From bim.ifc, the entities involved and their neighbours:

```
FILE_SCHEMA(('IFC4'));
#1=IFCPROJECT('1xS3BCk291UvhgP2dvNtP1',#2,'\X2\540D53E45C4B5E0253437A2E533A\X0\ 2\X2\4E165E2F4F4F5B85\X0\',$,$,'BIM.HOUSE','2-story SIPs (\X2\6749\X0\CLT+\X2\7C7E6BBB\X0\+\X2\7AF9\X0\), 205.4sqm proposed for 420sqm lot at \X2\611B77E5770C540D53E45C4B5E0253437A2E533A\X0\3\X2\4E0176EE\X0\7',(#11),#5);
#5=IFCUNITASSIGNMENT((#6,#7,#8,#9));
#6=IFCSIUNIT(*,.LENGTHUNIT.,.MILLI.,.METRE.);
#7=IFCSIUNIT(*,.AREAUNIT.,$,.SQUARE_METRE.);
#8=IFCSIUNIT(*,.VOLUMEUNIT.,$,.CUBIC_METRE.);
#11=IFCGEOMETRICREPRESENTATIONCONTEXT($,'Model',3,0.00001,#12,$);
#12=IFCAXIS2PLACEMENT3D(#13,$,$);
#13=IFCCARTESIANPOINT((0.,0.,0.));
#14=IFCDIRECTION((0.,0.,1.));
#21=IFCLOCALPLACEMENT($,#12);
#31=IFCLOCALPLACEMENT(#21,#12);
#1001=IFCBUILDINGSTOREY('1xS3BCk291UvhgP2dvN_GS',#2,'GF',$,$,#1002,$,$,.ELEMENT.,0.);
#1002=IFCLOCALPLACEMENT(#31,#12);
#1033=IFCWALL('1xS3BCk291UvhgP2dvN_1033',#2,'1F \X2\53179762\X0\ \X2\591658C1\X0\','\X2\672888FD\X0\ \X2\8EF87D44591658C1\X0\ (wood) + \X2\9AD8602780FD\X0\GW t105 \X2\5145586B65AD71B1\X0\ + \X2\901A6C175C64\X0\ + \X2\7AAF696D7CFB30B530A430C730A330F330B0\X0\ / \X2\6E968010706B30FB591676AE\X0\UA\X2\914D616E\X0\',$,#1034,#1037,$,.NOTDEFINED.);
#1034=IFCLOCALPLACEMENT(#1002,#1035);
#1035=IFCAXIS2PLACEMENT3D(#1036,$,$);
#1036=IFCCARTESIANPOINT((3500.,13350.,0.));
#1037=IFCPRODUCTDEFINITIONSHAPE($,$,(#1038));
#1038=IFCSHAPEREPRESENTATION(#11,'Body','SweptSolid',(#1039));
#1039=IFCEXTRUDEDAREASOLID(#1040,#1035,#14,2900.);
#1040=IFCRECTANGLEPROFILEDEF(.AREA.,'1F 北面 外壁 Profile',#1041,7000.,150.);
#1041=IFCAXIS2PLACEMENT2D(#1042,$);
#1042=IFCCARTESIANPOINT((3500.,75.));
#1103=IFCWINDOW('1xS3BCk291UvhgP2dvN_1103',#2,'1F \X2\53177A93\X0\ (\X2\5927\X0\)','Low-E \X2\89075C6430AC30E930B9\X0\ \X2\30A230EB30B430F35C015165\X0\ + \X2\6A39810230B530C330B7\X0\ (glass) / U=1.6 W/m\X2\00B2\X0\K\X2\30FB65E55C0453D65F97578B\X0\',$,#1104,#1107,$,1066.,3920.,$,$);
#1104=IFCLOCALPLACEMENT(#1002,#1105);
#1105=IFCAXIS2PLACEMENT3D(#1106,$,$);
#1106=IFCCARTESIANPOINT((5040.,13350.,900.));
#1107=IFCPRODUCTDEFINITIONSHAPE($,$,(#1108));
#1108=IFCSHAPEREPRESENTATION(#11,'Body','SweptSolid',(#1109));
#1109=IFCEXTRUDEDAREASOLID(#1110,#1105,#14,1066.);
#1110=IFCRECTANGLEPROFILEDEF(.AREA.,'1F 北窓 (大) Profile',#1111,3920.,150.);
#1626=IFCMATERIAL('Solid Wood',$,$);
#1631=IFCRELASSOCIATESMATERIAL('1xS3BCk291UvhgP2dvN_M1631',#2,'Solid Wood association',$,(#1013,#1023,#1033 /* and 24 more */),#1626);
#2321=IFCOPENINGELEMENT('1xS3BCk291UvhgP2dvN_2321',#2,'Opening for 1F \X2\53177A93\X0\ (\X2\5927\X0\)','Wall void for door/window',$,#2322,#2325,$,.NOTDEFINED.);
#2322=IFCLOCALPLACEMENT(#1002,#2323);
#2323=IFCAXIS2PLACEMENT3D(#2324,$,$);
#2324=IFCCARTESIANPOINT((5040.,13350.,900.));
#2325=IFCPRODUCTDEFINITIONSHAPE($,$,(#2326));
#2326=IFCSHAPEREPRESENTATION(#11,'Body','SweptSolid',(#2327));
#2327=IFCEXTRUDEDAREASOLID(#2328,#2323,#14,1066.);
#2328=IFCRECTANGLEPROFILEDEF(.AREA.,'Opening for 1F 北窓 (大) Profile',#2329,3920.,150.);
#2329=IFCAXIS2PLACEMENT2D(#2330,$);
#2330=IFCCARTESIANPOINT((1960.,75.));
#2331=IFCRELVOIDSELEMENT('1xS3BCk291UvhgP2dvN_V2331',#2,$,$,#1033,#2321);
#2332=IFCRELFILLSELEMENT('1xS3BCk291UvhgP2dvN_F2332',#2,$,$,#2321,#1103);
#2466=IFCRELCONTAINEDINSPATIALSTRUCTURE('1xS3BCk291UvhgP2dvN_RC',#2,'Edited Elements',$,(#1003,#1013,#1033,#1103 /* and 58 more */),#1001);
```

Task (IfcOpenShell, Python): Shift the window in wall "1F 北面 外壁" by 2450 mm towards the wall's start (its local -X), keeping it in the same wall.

```python
import ifcopenshell
import ifcopenshell.api.geometry
import ifcopenshell.util.placement
import ifcopenshell.util.unit

model = ifcopenshell.open("bim.ifc")
unit_scale = ifcopenshell.util.unit.calculate_unit_scale(model)

window = model.by_guid("1xS3BCk291UvhgP2dvN_1103")
opening = window.FillsVoids[0].RelatingOpeningElement
wall = opening.VoidsElements[0].RelatingBuildingElement

wall_matrix = ifcopenshell.util.placement.get_local_placement(wall.ObjectPlacement)
shift = wall_matrix[:3, 0] * -2.45 / unit_scale
before = ifcopenshell.util.placement.get_local_placement(window.ObjectPlacement)[:3, 3].copy()

# The window is not placed relative to its opening, so move both.
for product in (opening, window):
    matrix = ifcopenshell.util.placement.get_local_placement(product.ObjectPlacement)
    matrix[:3, 3] += shift
    ifcopenshell.api.geometry.edit_object_placement(model, product=product, matrix=matrix, is_si=False)

after = ifcopenshell.util.placement.get_local_placement(window.ObjectPlacement)[:3, 3]
print("window moved by", (after - before).round(3) + 0.0)

model.write("bim_v2.ifc")
```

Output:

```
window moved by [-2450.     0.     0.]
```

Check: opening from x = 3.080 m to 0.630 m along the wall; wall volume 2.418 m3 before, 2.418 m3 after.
